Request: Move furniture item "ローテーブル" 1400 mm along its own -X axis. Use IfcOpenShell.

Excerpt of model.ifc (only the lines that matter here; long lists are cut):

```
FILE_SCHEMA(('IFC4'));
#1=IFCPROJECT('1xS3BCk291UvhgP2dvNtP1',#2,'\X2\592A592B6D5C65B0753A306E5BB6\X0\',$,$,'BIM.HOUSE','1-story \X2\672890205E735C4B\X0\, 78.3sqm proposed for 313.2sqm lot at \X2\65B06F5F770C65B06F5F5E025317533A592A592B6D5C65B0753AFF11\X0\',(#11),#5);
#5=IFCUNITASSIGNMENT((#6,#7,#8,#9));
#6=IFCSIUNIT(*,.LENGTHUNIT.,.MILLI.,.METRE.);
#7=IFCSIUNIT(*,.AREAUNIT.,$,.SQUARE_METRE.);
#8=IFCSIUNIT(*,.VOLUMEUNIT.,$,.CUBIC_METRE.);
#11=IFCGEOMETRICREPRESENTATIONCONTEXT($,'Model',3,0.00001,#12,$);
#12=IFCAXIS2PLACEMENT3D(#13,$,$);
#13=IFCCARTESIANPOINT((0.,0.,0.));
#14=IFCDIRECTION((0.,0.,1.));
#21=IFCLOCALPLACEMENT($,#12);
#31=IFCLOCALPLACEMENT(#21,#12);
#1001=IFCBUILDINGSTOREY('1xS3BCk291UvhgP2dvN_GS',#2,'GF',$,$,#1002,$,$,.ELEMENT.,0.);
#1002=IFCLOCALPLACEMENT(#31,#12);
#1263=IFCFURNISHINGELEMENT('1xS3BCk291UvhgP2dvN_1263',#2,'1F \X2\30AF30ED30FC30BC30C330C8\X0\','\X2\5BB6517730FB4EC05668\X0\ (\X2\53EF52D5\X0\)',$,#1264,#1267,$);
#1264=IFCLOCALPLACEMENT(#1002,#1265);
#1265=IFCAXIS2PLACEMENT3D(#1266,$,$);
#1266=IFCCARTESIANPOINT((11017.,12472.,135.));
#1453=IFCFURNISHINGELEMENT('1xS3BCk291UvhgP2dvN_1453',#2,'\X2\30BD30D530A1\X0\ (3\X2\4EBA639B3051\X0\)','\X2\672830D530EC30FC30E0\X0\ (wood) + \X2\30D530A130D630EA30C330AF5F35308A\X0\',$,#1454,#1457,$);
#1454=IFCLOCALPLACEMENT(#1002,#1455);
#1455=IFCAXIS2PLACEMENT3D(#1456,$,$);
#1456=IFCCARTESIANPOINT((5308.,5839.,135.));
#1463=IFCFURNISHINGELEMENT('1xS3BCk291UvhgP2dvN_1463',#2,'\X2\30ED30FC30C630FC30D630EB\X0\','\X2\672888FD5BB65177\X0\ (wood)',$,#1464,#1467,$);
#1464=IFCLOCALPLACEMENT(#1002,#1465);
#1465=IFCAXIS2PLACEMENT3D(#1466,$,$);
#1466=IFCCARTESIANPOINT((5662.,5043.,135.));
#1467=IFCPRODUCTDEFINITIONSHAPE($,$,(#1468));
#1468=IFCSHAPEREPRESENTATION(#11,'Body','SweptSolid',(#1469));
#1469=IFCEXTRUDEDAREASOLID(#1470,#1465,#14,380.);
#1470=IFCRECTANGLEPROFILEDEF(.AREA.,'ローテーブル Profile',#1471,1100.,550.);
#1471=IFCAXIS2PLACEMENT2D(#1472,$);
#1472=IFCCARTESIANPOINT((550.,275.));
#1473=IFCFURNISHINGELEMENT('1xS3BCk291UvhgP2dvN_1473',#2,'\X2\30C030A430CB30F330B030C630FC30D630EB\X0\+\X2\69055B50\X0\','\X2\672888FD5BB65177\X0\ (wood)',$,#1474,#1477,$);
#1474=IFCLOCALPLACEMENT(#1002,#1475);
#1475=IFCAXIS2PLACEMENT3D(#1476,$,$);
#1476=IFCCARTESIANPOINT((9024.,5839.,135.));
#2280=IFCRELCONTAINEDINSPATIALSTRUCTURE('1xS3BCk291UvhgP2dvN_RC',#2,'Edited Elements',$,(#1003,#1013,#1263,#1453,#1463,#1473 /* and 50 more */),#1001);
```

```python
import ifcopenshell
import ifcopenshell.api.geometry
import ifcopenshell.util.placement
import ifcopenshell.util.unit

model = ifcopenshell.open("model.ifc")
unit_scale = ifcopenshell.util.unit.calculate_unit_scale(model)

item = model.by_id(1463)
matrix = ifcopenshell.util.placement.get_local_placement(item.ObjectPlacement)
matrix[:3, 3] -= matrix[:3, 0] * 1.4 / unit_scale
ifcopenshell.api.geometry.edit_object_placement(model, product=item, matrix=matrix, is_si=False)

print(ifcopenshell.util.placement.get_local_placement(item.ObjectPlacement).round(3) + 0.0)

model.write("model-out.ifc")
```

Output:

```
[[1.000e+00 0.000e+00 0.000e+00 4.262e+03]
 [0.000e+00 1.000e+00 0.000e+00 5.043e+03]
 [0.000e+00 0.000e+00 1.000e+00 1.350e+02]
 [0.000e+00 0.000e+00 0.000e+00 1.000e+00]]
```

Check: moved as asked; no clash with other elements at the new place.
